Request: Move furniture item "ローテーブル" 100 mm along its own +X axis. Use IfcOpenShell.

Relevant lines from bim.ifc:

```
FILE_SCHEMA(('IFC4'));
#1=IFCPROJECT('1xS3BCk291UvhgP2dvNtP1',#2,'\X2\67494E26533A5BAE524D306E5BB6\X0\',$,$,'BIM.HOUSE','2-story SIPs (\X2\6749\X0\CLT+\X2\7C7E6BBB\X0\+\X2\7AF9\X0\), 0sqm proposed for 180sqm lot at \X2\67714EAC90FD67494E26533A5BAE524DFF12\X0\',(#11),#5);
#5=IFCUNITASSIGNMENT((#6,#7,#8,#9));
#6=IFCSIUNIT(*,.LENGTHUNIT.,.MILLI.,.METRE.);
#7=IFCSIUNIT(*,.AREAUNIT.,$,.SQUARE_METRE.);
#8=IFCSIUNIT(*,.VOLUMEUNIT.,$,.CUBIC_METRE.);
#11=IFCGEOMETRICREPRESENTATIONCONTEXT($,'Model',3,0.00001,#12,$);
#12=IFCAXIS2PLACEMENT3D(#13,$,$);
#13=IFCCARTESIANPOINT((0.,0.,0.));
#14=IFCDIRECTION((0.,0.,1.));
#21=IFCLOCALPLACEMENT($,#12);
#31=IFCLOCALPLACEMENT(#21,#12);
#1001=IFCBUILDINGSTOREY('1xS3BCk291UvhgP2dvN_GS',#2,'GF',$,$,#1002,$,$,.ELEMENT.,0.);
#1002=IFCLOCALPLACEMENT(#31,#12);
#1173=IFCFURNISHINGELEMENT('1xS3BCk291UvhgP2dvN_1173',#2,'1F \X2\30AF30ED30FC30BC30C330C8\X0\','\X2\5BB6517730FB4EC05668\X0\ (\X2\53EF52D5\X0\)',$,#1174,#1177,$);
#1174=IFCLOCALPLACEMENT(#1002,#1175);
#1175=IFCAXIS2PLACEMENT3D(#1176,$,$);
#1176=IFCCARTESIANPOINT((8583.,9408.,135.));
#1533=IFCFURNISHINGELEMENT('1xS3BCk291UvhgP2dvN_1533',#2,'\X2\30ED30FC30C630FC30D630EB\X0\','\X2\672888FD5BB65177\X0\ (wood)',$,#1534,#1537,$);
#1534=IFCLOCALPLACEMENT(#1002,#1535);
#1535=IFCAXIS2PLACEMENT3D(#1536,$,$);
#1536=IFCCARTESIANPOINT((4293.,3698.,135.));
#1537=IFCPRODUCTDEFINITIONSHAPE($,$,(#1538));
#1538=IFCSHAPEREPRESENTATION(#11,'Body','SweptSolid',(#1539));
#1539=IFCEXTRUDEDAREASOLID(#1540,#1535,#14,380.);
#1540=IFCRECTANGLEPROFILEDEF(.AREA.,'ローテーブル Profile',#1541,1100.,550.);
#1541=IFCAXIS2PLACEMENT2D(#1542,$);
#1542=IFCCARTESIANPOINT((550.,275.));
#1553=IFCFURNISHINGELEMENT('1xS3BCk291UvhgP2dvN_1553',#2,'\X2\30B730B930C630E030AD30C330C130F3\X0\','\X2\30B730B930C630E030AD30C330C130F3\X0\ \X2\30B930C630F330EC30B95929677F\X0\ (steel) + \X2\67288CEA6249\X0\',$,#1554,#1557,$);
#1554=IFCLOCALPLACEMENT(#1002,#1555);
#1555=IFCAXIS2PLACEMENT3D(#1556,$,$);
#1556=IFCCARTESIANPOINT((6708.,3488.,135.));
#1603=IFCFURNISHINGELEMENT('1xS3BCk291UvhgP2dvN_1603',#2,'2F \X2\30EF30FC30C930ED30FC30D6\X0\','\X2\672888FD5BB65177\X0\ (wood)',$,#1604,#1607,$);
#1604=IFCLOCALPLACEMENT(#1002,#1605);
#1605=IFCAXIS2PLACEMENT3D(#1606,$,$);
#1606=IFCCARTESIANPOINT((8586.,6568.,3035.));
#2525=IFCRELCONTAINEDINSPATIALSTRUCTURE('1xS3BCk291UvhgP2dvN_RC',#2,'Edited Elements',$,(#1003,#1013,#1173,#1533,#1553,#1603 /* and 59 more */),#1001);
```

```python
import ifcopenshell
import ifcopenshell.api.geometry
import ifcopenshell.util.placement
import ifcopenshell.util.unit

model = ifcopenshell.open("bim.ifc")
unit_scale = ifcopenshell.util.unit.calculate_unit_scale(model)

item = model.by_guid("1xS3BCk291UvhgP2dvN_1533")
matrix = ifcopenshell.util.placement.get_local_placement(item.ObjectPlacement)
matrix[:3, 3] += matrix[:3, 0] * 0.1 / unit_scale
ifcopenshell.api.geometry.edit_object_placement(model, product=item, matrix=matrix, is_si=False)

print(ifcopenshell.util.placement.get_local_placement(item.ObjectPlacement).round(3) + 0.0)

model.write("bim_v2.ifc")
```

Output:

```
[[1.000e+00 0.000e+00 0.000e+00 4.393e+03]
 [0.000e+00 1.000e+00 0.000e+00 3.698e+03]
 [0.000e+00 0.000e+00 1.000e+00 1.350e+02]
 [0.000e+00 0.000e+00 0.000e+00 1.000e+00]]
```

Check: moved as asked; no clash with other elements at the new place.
